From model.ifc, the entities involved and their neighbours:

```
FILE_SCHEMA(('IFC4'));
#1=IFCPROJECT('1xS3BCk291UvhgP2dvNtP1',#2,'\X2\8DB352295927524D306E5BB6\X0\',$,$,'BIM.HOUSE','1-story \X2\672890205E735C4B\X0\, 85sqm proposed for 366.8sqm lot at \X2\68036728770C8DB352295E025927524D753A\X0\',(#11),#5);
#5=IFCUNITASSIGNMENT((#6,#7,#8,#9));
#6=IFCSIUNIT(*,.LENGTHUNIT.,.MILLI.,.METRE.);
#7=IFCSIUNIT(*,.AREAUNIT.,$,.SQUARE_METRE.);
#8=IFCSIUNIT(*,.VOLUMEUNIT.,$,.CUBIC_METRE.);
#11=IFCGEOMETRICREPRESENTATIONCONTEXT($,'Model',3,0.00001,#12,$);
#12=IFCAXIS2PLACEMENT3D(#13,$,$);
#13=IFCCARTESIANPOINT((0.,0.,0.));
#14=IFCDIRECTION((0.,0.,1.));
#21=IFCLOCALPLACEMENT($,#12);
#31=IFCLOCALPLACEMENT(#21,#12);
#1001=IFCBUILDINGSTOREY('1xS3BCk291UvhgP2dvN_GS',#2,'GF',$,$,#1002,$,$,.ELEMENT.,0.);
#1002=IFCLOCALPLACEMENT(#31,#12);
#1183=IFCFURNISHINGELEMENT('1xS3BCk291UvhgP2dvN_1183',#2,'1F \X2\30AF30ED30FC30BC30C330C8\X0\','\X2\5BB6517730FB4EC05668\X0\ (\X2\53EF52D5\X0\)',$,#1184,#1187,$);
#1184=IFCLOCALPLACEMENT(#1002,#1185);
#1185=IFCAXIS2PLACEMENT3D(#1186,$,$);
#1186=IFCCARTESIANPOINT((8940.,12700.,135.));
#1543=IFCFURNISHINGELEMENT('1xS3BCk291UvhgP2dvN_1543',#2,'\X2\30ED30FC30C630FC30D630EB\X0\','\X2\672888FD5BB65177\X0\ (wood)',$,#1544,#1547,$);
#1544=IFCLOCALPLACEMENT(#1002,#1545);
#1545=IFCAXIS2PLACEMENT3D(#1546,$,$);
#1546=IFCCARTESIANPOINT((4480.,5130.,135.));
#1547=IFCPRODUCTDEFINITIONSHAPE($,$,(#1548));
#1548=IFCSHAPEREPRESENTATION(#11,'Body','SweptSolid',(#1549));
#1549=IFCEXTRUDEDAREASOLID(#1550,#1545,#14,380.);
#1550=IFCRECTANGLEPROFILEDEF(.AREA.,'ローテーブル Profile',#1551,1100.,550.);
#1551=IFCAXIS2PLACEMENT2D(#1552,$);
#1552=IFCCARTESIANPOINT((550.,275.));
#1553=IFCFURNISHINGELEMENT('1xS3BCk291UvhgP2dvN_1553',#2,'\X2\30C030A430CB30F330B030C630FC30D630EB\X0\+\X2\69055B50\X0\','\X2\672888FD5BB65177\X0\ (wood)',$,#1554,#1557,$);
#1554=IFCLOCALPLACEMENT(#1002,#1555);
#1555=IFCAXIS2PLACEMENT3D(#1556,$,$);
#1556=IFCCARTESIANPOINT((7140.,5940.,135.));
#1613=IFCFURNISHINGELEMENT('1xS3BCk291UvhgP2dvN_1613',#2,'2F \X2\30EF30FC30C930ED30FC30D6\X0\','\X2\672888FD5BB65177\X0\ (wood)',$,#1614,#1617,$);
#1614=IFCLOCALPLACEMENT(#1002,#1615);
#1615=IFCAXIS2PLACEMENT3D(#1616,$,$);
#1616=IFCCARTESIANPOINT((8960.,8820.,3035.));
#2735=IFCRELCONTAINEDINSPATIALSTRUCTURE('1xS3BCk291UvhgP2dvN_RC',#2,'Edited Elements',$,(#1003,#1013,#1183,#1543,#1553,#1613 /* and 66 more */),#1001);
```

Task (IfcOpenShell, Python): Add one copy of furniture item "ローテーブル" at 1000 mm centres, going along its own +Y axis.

```python
import ifcopenshell
import ifcopenshell.api.geometry
import ifcopenshell.api.root
import ifcopenshell.util.element
import ifcopenshell.util.placement
import ifcopenshell.util.unit

model = ifcopenshell.open("model.ifc")
unit_scale = ifcopenshell.util.unit.calculate_unit_scale(model)


def reuse_history(source, copy):
    """copy_class also copies each property set's owner history, people and application; keep the originals."""
    for rel in copy.IsDefinedBy:
        if rel.is_a("IfcRelDefinesByProperties") and (history := rel.RelatingPropertyDefinition.OwnerHistory):
            rel.RelatingPropertyDefinition.OwnerHistory = source.OwnerHistory
            ifcopenshell.util.element.remove_deep2(model, history)


source = model.by_guid("1xS3BCk291UvhgP2dvN_1543")
base = ifcopenshell.util.placement.get_local_placement(source.ObjectPlacement)
step = base[:3, 1] * 1 / unit_scale

for i in range(1, 2):
    copy = ifcopenshell.api.root.copy_class(model, product=source)
    copy.Representation = ifcopenshell.util.element.copy_deep(
        model, source.Representation, exclude=["IfcGeometricRepresentationContext", "IfcRepresentationMap"]
    )
    reuse_history(source, copy)
    matrix = base.copy()
    matrix[:3, 3] += i * step
    print("added at", matrix[:3, 3].round(3) + 0.0)
    ifcopenshell.api.geometry.edit_object_placement(model, product=copy, matrix=matrix, is_si=False)

model.write("model_v2.ifc")
```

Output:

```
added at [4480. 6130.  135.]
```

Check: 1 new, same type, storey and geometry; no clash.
